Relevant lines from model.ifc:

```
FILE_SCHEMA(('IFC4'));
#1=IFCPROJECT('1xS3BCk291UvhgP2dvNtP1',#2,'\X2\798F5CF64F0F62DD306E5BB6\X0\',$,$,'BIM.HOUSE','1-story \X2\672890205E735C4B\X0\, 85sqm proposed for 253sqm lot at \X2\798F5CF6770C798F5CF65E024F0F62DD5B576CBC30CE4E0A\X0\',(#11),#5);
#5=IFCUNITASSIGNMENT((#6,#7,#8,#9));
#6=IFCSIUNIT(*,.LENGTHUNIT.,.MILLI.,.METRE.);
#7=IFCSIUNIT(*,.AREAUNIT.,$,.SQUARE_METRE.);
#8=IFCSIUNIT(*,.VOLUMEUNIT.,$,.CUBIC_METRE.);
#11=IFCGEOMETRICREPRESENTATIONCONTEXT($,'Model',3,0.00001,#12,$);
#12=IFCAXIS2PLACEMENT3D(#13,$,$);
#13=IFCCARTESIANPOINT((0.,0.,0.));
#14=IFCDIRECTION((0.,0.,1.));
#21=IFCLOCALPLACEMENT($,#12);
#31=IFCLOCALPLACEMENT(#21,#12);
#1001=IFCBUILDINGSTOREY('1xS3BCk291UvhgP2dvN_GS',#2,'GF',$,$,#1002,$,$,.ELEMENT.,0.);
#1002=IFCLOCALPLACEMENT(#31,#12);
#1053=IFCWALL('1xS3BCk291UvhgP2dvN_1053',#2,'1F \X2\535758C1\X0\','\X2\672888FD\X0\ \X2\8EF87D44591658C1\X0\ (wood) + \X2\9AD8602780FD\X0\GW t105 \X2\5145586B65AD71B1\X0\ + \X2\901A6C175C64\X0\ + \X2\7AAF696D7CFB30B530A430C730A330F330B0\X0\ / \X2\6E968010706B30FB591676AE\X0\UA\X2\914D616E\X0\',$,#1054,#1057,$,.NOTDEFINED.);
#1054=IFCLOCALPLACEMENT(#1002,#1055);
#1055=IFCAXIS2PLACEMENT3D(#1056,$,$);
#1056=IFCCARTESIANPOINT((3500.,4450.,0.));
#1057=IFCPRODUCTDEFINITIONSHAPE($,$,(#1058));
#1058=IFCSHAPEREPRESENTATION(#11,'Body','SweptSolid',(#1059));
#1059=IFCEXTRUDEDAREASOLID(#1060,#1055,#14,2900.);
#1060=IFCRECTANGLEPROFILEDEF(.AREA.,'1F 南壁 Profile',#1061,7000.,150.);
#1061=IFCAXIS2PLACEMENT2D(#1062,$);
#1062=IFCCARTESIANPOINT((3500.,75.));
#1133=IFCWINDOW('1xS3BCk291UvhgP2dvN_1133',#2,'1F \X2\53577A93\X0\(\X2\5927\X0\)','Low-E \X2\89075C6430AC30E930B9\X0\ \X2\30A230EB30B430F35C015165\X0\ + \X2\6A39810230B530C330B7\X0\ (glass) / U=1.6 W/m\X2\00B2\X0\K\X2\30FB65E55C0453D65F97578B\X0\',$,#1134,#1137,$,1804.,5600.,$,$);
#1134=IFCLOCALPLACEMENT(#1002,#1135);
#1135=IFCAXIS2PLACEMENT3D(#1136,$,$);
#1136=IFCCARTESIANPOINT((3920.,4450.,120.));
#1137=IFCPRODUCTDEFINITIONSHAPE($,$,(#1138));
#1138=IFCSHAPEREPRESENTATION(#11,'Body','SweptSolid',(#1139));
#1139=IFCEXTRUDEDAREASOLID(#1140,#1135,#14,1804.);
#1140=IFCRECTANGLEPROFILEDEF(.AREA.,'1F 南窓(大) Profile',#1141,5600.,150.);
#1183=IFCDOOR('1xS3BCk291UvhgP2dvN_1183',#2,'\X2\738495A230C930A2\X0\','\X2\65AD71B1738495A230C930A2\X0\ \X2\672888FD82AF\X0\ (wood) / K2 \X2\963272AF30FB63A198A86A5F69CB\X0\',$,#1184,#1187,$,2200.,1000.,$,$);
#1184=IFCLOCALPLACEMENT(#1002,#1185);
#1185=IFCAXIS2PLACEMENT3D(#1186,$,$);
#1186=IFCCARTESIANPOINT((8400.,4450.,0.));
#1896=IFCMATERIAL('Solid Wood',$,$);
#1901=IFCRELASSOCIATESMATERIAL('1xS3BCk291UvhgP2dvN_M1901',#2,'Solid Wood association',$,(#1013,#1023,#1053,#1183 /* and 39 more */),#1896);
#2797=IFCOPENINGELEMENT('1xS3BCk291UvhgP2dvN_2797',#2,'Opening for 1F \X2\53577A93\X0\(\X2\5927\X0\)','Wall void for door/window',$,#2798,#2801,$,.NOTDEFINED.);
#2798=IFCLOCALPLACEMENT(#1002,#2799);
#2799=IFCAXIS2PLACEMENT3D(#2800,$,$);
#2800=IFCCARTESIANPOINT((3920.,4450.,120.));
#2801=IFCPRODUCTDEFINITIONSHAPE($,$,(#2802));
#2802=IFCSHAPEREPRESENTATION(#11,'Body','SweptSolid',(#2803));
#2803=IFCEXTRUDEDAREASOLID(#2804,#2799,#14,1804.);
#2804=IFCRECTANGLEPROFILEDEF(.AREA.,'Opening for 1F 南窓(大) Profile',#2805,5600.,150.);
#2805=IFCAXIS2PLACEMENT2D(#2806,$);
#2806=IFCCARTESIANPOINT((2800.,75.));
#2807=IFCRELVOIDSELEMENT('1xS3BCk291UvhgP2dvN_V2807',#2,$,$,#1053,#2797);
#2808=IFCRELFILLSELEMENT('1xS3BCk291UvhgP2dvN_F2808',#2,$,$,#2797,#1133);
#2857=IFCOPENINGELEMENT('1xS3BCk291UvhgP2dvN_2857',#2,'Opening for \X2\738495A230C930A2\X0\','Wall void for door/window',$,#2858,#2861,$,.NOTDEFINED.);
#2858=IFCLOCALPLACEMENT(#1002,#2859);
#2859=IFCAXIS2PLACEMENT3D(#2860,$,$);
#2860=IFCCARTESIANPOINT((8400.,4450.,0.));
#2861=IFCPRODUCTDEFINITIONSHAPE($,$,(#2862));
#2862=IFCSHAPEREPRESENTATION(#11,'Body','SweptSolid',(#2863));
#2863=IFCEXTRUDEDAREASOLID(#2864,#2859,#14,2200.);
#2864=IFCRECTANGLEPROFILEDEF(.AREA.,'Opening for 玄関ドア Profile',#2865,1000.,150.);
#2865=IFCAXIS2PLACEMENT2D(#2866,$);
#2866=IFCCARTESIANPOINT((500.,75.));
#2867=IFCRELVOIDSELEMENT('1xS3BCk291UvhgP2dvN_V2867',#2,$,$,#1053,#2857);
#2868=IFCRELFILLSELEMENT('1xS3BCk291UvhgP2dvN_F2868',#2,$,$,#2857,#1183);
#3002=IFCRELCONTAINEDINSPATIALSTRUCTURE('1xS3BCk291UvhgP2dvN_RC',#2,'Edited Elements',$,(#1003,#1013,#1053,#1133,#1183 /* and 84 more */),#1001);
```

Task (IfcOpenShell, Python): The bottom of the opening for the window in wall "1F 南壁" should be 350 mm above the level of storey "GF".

```python
import numpy as np
import ifcopenshell
import ifcopenshell.api.geometry
import ifcopenshell.geom
import ifcopenshell.util.element
import ifcopenshell.util.placement
import ifcopenshell.util.shape
import ifcopenshell.util.unit

model = ifcopenshell.open("model.ifc")
unit_scale = ifcopenshell.util.unit.calculate_unit_scale(model)

window = model.by_guid("1xS3BCk291UvhgP2dvN_1133")
opening = window.FillsVoids[0].RelatingOpeningElement
storey = ifcopenshell.util.element.get_container(window, ifc_class="IfcBuildingStorey")
level = ifcopenshell.util.placement.get_local_placement(storey.ObjectPlacement)[2, 3]

# The opening's origin need not be at the sill, so measure its lowest point.
shape = ifcopenshell.geom.create_shape(ifcopenshell.geom.settings(), opening)
bottom = ifcopenshell.util.shape.get_shape_bottom_elevation(shape, shape.geometry) / unit_scale
dz = level + 350.0 - bottom

shift = np.array([0.0, 0.0, dz])
# The window is not placed relative to its opening, so move both.
for product in (opening, window):
    matrix = ifcopenshell.util.placement.get_local_placement(product.ObjectPlacement)
    matrix[:3, 3] += shift
    ifcopenshell.api.geometry.edit_object_placement(model, product=product, matrix=matrix, is_si=False)

print(f"moved by {dz * unit_scale:+.3f} m")

model.write("model-out.ifc")
```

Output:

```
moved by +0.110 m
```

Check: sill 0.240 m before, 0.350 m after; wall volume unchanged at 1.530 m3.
